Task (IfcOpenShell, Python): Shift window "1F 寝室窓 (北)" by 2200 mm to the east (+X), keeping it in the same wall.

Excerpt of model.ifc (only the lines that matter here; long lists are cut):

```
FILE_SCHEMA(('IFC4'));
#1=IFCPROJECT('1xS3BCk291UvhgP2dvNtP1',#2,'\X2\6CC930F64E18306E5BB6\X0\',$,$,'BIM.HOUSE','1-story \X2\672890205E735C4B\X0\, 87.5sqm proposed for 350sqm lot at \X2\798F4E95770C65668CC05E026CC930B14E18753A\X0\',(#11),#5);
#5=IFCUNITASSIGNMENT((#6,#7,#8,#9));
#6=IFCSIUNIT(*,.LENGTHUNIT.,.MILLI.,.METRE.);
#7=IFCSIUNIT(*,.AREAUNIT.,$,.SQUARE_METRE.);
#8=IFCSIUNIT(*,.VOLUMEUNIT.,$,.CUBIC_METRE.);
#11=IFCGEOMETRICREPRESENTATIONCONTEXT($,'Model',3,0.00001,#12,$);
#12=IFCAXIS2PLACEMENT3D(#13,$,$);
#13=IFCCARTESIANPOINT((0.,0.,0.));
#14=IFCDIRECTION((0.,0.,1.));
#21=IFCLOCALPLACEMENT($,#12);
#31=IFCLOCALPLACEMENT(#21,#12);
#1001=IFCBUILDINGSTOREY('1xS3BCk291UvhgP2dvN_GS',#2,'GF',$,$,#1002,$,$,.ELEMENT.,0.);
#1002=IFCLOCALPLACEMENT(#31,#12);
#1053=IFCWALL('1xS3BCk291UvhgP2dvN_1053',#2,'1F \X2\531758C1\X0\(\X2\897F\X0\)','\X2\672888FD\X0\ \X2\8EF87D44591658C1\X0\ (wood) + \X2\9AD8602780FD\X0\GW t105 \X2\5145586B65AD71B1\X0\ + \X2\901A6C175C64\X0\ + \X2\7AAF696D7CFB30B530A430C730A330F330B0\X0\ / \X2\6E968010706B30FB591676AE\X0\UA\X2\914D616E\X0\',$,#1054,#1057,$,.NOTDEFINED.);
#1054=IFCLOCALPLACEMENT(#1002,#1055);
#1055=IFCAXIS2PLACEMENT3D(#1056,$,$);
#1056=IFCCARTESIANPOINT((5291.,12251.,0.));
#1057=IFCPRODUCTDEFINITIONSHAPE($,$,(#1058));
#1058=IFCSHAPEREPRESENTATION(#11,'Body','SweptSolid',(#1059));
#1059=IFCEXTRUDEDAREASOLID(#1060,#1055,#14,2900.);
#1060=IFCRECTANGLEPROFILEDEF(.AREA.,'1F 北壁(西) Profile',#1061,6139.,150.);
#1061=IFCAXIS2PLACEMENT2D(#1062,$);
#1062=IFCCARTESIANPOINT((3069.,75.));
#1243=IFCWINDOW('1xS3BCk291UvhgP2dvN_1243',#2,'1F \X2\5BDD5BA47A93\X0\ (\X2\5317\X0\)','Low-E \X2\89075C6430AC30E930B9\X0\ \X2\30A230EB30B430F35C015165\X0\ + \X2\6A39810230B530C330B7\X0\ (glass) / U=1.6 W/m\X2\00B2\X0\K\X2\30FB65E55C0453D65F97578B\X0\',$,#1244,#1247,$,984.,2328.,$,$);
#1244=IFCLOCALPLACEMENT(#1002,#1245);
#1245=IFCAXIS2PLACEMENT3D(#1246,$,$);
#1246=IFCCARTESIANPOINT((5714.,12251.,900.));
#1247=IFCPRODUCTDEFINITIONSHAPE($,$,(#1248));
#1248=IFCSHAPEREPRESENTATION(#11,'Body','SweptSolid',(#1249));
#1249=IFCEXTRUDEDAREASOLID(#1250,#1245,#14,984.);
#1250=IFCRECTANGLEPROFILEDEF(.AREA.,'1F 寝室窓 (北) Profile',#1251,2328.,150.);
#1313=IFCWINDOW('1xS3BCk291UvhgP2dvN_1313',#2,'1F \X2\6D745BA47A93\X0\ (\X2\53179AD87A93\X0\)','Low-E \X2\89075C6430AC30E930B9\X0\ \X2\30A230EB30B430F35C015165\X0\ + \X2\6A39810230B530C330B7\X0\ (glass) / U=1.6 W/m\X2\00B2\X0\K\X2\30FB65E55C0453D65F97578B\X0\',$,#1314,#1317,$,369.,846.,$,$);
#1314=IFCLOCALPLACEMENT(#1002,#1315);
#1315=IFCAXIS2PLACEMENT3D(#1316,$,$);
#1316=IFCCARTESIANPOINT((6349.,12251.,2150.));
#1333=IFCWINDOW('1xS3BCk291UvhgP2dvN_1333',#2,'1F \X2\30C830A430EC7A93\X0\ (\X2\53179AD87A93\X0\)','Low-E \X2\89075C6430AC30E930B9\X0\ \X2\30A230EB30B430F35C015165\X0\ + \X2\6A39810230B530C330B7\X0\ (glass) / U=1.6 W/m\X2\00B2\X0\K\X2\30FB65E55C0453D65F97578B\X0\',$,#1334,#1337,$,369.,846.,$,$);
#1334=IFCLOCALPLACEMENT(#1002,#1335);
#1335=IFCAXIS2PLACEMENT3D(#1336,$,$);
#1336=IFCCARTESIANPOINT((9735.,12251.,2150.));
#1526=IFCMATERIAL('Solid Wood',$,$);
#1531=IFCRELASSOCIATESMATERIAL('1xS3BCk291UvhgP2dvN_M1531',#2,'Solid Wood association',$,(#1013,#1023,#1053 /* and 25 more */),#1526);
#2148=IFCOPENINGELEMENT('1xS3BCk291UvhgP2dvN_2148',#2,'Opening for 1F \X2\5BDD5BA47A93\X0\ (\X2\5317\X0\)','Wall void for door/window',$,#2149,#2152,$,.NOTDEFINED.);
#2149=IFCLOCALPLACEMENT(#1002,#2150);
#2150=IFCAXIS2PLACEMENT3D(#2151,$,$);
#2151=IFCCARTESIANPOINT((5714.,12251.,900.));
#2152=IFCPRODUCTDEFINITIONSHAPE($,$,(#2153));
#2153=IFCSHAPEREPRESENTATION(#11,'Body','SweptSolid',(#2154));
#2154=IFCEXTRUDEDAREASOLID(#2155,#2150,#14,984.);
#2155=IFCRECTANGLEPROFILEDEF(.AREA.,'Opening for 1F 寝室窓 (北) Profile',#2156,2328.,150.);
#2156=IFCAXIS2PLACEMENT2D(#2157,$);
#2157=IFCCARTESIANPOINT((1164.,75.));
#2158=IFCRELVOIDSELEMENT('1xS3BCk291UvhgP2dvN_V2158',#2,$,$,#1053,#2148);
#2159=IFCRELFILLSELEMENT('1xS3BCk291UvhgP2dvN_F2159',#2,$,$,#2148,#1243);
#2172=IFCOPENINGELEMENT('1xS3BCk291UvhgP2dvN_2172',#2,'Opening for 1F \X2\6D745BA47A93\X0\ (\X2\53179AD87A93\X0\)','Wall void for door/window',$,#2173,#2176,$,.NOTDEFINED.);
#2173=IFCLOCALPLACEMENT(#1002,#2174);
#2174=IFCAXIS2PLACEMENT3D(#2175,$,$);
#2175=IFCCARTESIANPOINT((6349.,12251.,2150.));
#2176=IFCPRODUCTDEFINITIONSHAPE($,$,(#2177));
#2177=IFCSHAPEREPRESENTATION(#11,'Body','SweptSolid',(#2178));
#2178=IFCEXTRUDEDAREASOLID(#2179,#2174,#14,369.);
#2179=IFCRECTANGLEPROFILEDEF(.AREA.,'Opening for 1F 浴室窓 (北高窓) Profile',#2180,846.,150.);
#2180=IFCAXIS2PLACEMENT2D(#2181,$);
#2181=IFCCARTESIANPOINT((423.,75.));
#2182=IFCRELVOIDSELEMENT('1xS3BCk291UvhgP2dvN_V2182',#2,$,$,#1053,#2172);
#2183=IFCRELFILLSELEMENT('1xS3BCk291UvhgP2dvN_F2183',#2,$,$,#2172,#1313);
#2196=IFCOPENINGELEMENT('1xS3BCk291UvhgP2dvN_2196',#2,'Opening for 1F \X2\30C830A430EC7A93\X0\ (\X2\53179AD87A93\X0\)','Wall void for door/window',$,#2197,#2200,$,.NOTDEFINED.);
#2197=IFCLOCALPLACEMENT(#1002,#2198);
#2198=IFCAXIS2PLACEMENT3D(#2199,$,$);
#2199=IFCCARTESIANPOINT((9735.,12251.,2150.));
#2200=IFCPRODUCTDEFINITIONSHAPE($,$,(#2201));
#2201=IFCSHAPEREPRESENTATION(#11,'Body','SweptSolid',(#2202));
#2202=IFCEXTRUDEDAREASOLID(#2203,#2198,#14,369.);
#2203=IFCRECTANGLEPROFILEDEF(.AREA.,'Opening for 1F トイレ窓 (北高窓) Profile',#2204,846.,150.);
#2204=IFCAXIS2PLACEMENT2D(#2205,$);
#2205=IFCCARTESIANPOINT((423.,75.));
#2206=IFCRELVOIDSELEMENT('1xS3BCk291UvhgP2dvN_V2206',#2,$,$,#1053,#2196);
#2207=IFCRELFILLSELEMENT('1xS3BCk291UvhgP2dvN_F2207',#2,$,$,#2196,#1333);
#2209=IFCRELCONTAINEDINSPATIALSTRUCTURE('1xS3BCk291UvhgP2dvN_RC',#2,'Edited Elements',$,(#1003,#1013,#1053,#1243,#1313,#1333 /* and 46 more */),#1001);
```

```python
import ifcopenshell
import ifcopenshell.api.geometry
import ifcopenshell.util.placement
import ifcopenshell.util.unit

model = ifcopenshell.open("model.ifc")
unit_scale = ifcopenshell.util.unit.calculate_unit_scale(model)

window = model.by_guid("1xS3BCk291UvhgP2dvN_1243")
opening = window.FillsVoids[0].RelatingOpeningElement
wall = opening.VoidsElements[0].RelatingBuildingElement

wall_matrix = ifcopenshell.util.placement.get_local_placement(wall.ObjectPlacement)
shift = wall_matrix[:3, 0] * 2.2 / unit_scale
before = ifcopenshell.util.placement.get_local_placement(window.ObjectPlacement)[:3, 3].copy()

# The window is not placed relative to its opening, so move both.
for product in (opening, window):
    matrix = ifcopenshell.util.placement.get_local_placement(product.ObjectPlacement)
    matrix[:3, 3] += shift
    ifcopenshell.api.geometry.edit_object_placement(model, product=product, matrix=matrix, is_si=False)

after = ifcopenshell.util.placement.get_local_placement(window.ObjectPlacement)[:3, 3]
print("window moved by", (after - before).round(3) + 0.0)

model.write("model-out.ifc")
```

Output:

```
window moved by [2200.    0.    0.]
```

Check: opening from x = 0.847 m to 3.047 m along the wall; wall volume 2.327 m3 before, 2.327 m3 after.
